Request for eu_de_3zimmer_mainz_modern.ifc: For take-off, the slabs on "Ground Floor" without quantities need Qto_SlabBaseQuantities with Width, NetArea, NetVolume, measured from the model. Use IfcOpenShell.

First a look at what the model holds.

```python
import ifcopenshell
import ifcopenshell.util.element
import ifcopenshell.util.unit

model = ifcopenshell.open("eu_de_3zimmer_mainz_modern.ifc")
print(model.schema)
for unit_type in ("LENGTHUNIT", "AREAUNIT", "VOLUMEUNIT"):
    print(unit_type, ifcopenshell.util.unit.calculate_unit_scale(model, unit_type))
storey = next(s for s in model.by_type("IfcBuildingStorey") if s.Name == "Ground Floor")
slabs = [e for e in ifcopenshell.util.element.get_decomposition(storey) if e.is_a("IfcSlab")]
for e in sorted(slabs, key=lambda e: e.id()):
    print(e.id(), e.is_a(), e.Name, list(ifcopenshell.util.element.get_psets(e, qtos_only=True)), sep=" | ")
```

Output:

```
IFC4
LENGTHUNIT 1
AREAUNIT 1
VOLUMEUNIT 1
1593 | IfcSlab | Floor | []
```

```python
import ifcopenshell
import ifcopenshell.api.pset
import ifcopenshell.geom
import ifcopenshell.util.element
import ifcopenshell.util.shape
import ifcopenshell.util.unit

model = ifcopenshell.open("eu_de_3zimmer_mainz_modern.ifc")
unit_scale = ifcopenshell.util.unit.calculate_unit_scale(model)
area_scale = ifcopenshell.util.unit.calculate_unit_scale(model, "AREAUNIT")
volume_scale = ifcopenshell.util.unit.calculate_unit_scale(model, "VOLUMEUNIT")
settings = ifcopenshell.geom.settings()

storey = next(s for s in model.by_type("IfcBuildingStorey") if s.Name == "Ground Floor")
slabs = [e for e in ifcopenshell.util.element.get_decomposition(storey) if e.is_a("IfcSlab")]

for e in sorted(slabs, key=lambda e: e.id()):
    if ifcopenshell.util.element.get_psets(e, qtos_only=True, should_inherit=False):
        continue
    # Geometry comes back in metres, in the element's own axes.
    shape = ifcopenshell.geom.create_shape(settings, e)
    values = {
        "Width": ifcopenshell.util.shape.get_z(shape.geometry) / unit_scale,
        "NetArea": ifcopenshell.util.shape.get_footprint_area(shape.geometry) / area_scale,
        "NetVolume": ifcopenshell.util.shape.get_volume(shape.geometry) / volume_scale,
    }
    qto = ifcopenshell.api.pset.add_qto(model, product=e, name="Qto_SlabBaseQuantities")
    ifcopenshell.api.pset.edit_qto(model, qto=qto, properties=values)
    print(e.id(), {k: round(v, 3) for k, v in values.items()})

model.write("eu_de_3zimmer_mainz_modern-out.ifc")
```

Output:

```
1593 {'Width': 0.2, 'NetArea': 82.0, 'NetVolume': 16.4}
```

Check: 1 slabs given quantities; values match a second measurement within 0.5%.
